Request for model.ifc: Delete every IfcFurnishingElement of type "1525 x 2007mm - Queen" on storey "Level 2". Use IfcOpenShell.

First a look at what the model holds.

```python
import ifcopenshell
import ifcopenshell.util.element

model = ifcopenshell.open("model.ifc")
print(model.schema)
storey = next(s for s in model.by_type("IfcBuildingStorey") if s.Name == "Level 2")
furniture = [e for e in ifcopenshell.util.element.get_decomposition(storey) if e.is_a("IfcFurnishingElement")]
seen = {}
for e in furniture:
    element_type = ifcopenshell.util.element.get_type(e)
    name = element_type.Name if element_type not in (None, e) else None
    seen[name] = seen.get(name, 0) + 1
for name, count in sorted(seen.items(), key=str):
    print(count, "x", name)
```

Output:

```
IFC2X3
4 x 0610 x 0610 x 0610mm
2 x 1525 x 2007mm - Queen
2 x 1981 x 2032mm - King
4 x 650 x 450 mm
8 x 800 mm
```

```python
import ifcopenshell
import ifcopenshell.api.root
import ifcopenshell.util.element

model = ifcopenshell.open("model.ifc")

storey = next(s for s in model.by_type("IfcBuildingStorey") if s.Name == "Level 2")
furniture = [e for e in ifcopenshell.util.element.get_decomposition(storey) if e.is_a("IfcFurnishingElement")]
targets = [e for e in furniture if (t := ifcopenshell.util.element.get_type(e)) not in (None, e) and t.Name == "1525 x 2007mm - Queen"]

for e in targets:
    ifcopenshell.api.root.remove_product(model, product=e)
print(len(targets), "removed")

model.write("model_updated.ifc")
```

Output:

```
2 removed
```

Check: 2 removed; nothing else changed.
